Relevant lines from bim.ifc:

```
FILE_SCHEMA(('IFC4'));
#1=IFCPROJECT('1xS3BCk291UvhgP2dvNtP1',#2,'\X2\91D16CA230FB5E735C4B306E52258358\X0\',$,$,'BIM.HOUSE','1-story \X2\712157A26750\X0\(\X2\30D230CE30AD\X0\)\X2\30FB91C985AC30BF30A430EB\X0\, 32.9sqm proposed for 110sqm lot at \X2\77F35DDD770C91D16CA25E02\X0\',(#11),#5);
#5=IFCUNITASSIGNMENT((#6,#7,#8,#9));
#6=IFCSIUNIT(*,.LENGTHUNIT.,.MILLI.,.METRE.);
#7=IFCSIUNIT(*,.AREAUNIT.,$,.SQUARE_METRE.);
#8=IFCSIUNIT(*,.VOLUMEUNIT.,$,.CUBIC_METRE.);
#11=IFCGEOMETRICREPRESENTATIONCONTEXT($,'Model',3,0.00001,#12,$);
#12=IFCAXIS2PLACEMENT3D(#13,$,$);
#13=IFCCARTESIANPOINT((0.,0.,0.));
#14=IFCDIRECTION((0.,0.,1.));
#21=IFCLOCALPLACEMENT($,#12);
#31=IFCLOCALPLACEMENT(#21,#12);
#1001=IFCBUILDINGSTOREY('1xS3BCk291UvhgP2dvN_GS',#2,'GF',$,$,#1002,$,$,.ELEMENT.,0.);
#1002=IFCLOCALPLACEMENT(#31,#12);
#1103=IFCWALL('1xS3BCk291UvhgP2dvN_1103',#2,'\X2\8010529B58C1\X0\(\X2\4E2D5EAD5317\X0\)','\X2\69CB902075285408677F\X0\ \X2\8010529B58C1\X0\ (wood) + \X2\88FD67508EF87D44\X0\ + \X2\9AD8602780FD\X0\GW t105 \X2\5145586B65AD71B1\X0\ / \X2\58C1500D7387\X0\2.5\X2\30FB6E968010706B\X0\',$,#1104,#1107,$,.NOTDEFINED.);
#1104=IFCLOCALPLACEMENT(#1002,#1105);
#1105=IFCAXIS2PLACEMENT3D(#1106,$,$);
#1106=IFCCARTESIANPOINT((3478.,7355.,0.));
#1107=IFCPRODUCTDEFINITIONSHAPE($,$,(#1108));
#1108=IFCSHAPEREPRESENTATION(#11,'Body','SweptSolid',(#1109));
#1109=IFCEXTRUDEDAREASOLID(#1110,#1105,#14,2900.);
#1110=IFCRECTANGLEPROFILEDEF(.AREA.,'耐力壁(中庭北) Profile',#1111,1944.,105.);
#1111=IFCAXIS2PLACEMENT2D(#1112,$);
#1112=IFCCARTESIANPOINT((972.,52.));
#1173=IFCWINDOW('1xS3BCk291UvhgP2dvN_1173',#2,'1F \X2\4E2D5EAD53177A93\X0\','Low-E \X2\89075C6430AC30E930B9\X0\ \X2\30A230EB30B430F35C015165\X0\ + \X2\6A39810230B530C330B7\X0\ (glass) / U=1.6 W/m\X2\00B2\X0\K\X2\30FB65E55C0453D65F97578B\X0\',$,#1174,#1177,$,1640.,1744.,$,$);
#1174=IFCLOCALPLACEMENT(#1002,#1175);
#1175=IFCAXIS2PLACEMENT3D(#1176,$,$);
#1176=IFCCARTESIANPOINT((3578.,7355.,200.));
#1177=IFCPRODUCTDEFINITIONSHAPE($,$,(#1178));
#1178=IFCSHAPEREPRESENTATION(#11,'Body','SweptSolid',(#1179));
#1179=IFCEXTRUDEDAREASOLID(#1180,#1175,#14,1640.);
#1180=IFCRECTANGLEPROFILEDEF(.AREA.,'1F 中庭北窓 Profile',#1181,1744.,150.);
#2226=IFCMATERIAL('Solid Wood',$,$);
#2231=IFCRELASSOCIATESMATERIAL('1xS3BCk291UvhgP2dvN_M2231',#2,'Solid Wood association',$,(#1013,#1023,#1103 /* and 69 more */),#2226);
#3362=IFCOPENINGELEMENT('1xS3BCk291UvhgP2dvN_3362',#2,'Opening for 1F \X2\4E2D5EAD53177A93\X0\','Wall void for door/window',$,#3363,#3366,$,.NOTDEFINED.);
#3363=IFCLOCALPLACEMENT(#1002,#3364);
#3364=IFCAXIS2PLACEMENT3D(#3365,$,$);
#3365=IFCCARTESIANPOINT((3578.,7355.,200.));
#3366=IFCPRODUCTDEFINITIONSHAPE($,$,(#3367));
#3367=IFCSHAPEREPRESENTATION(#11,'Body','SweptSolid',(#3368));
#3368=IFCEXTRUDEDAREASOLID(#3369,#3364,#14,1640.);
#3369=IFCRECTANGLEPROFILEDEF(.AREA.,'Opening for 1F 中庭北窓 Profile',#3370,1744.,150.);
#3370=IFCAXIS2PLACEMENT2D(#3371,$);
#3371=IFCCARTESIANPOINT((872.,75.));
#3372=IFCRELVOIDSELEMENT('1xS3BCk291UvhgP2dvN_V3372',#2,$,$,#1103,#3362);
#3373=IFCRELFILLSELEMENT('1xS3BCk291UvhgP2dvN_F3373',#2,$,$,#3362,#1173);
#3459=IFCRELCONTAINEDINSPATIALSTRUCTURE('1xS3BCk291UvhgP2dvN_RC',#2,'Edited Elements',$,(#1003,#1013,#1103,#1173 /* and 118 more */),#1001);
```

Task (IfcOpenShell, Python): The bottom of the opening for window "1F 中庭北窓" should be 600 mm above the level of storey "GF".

```python
import numpy as np
import ifcopenshell
import ifcopenshell.api.geometry
import ifcopenshell.geom
import ifcopenshell.util.element
import ifcopenshell.util.placement
import ifcopenshell.util.shape
import ifcopenshell.util.unit

model = ifcopenshell.open("bim.ifc")
unit_scale = ifcopenshell.util.unit.calculate_unit_scale(model)

window = model.by_guid("1xS3BCk291UvhgP2dvN_1173")
opening = window.FillsVoids[0].RelatingOpeningElement
storey = ifcopenshell.util.element.get_container(window, ifc_class="IfcBuildingStorey")
level = ifcopenshell.util.placement.get_local_placement(storey.ObjectPlacement)[2, 3]

# The opening's origin need not be at the sill, so measure its lowest point.
shape = ifcopenshell.geom.create_shape(ifcopenshell.geom.settings(), opening)
bottom = ifcopenshell.util.shape.get_shape_bottom_elevation(shape, shape.geometry) / unit_scale
dz = level + 0.6 / unit_scale - bottom

shift = np.array([0.0, 0.0, dz])
# The window is not placed relative to its opening, so move both.
for product in (opening, window):
    matrix = ifcopenshell.util.placement.get_local_placement(product.ObjectPlacement)
    matrix[:3, 3] += shift
    ifcopenshell.api.geometry.edit_object_placement(model, product=product, matrix=matrix, is_si=False)

print(f"moved by {dz * unit_scale:+.3f} m")

model.write("bim_v2.ifc")
```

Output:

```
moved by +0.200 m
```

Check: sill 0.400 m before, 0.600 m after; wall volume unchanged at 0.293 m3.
